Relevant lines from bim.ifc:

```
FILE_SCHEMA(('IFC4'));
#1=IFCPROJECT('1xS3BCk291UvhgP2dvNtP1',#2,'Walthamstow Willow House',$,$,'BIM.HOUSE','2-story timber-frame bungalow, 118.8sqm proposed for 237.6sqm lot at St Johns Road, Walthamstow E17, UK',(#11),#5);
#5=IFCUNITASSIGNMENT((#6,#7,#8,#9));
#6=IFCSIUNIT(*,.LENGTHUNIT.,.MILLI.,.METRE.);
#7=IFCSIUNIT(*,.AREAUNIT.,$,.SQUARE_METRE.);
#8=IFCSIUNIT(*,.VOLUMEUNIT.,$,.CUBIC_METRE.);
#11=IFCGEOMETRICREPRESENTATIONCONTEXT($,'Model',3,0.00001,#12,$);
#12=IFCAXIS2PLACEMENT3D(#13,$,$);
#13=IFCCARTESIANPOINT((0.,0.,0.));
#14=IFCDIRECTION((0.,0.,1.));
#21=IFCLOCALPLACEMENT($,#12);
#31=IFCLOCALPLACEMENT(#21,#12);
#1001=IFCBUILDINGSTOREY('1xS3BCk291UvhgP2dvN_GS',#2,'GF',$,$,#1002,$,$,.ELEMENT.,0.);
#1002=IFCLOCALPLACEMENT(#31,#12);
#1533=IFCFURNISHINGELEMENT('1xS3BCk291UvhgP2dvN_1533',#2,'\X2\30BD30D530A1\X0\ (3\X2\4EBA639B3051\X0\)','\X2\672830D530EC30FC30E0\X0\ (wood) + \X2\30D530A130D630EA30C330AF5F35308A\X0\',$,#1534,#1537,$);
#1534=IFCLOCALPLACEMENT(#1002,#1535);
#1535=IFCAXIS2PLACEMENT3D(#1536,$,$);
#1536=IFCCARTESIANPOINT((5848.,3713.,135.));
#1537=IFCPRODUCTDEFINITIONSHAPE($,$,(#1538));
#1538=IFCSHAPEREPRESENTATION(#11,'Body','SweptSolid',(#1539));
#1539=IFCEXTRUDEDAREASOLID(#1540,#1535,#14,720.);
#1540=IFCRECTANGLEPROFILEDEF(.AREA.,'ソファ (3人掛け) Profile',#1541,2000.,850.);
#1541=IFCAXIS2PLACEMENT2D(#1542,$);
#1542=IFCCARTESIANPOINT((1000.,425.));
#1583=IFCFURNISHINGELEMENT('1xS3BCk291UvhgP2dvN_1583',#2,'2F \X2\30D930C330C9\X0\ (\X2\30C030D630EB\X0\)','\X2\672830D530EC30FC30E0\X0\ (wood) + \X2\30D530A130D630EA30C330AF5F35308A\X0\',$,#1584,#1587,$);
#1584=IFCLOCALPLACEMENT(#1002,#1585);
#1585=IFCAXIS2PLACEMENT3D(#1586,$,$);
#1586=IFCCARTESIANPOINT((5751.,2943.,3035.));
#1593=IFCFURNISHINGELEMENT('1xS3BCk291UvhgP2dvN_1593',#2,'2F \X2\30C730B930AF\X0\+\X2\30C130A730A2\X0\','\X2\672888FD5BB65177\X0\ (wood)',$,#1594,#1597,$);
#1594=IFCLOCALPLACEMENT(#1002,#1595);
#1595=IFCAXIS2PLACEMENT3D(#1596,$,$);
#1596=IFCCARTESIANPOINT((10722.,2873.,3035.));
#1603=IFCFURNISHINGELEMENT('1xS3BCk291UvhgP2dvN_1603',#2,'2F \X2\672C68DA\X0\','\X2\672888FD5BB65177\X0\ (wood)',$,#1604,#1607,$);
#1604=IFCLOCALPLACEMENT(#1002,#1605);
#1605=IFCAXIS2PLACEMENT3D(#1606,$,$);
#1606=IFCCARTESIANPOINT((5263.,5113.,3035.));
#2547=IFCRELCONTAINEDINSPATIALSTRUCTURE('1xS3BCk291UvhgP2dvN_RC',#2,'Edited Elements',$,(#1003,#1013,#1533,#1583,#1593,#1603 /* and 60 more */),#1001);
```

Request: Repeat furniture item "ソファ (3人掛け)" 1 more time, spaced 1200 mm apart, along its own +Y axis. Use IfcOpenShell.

```python
import ifcopenshell
import ifcopenshell.api.geometry
import ifcopenshell.api.root
import ifcopenshell.util.element
import ifcopenshell.util.placement

model = ifcopenshell.open("bim.ifc")


def reuse_history(source, copy):
    """copy_class also copies each property set's owner history, people and application; keep the originals."""
    for rel in copy.IsDefinedBy:
        if rel.is_a("IfcRelDefinesByProperties") and (history := rel.RelatingPropertyDefinition.OwnerHistory):
            rel.RelatingPropertyDefinition.OwnerHistory = source.OwnerHistory
            ifcopenshell.util.element.remove_deep2(model, history)


source = model.by_guid("1xS3BCk291UvhgP2dvN_1533")
base = ifcopenshell.util.placement.get_local_placement(source.ObjectPlacement)
step = base[:3, 1] * 1200.0

for i in range(1, 2):
    copy = ifcopenshell.api.root.copy_class(model, product=source)
    copy.Representation = ifcopenshell.util.element.copy_deep(
        model, source.Representation, exclude=["IfcGeometricRepresentationContext", "IfcRepresentationMap"]
    )
    reuse_history(source, copy)
    matrix = base.copy()
    matrix[:3, 3] += i * step
    print("added at", matrix[:3, 3].round(3) + 0.0)
    ifcopenshell.api.geometry.edit_object_placement(model, product=copy, matrix=matrix, is_si=False)

model.write("bim-out.ifc")
```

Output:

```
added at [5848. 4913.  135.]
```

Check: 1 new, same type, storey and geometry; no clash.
